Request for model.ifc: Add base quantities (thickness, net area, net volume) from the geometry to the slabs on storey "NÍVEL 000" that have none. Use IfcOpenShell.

First a look at what the model holds.

```python
import ifcopenshell
import ifcopenshell.util.element
import ifcopenshell.util.unit

model = ifcopenshell.open("model.ifc")
print(model.schema)
for unit_type in ("LENGTHUNIT", "AREAUNIT", "VOLUMEUNIT"):
    print(unit_type, ifcopenshell.util.unit.calculate_unit_scale(model, unit_type))
storey = next(s for s in model.by_type("IfcBuildingStorey") if s.Name == "NÍVEL 000")
slabs = [e for e in ifcopenshell.util.element.get_decomposition(storey) if e.is_a("IfcSlab")]
for e in sorted(slabs, key=lambda e: e.id()):
    print(e.id(), e.is_a(), e.Name, list(ifcopenshell.util.element.get_psets(e, qtos_only=True)), sep=" | ")
```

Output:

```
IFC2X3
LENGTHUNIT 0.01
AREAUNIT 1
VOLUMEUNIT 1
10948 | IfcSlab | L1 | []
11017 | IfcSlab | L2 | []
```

```python
import ifcopenshell
import ifcopenshell.api.pset
import ifcopenshell.geom
import ifcopenshell.util.element
import ifcopenshell.util.shape
import ifcopenshell.util.unit

model = ifcopenshell.open("model.ifc")
unit_scale = ifcopenshell.util.unit.calculate_unit_scale(model)
area_scale = ifcopenshell.util.unit.calculate_unit_scale(model, "AREAUNIT")
volume_scale = ifcopenshell.util.unit.calculate_unit_scale(model, "VOLUMEUNIT")
settings = ifcopenshell.geom.settings()

storey = next(s for s in model.by_type("IfcBuildingStorey") if s.Name == "NÍVEL 000")
slabs = [e for e in ifcopenshell.util.element.get_decomposition(storey) if e.is_a("IfcSlab")]

for e in sorted(slabs, key=lambda e: e.id()):
    if ifcopenshell.util.element.get_psets(e, qtos_only=True, should_inherit=False):
        continue
    # Geometry comes back in metres, in the element's own axes.
    shape = ifcopenshell.geom.create_shape(settings, e)
    values = {
        "Width": ifcopenshell.util.shape.get_z(shape.geometry) / unit_scale,
        "NetArea": ifcopenshell.util.shape.get_footprint_area(shape.geometry) / area_scale,
        "NetVolume": ifcopenshell.util.shape.get_volume(shape.geometry) / volume_scale,
    }
    qto = ifcopenshell.api.pset.add_qto(model, product=e, name="BaseQuantities")
    ifcopenshell.api.pset.edit_qto(model, qto=qto, properties=values)
    print(e.id(), {k: round(v, 3) for k, v in values.items()})

model.write("model_updated.ifc")
```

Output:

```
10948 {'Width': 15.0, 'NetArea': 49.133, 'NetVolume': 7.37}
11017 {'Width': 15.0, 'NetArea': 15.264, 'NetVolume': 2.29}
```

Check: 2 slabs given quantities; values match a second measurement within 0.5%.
